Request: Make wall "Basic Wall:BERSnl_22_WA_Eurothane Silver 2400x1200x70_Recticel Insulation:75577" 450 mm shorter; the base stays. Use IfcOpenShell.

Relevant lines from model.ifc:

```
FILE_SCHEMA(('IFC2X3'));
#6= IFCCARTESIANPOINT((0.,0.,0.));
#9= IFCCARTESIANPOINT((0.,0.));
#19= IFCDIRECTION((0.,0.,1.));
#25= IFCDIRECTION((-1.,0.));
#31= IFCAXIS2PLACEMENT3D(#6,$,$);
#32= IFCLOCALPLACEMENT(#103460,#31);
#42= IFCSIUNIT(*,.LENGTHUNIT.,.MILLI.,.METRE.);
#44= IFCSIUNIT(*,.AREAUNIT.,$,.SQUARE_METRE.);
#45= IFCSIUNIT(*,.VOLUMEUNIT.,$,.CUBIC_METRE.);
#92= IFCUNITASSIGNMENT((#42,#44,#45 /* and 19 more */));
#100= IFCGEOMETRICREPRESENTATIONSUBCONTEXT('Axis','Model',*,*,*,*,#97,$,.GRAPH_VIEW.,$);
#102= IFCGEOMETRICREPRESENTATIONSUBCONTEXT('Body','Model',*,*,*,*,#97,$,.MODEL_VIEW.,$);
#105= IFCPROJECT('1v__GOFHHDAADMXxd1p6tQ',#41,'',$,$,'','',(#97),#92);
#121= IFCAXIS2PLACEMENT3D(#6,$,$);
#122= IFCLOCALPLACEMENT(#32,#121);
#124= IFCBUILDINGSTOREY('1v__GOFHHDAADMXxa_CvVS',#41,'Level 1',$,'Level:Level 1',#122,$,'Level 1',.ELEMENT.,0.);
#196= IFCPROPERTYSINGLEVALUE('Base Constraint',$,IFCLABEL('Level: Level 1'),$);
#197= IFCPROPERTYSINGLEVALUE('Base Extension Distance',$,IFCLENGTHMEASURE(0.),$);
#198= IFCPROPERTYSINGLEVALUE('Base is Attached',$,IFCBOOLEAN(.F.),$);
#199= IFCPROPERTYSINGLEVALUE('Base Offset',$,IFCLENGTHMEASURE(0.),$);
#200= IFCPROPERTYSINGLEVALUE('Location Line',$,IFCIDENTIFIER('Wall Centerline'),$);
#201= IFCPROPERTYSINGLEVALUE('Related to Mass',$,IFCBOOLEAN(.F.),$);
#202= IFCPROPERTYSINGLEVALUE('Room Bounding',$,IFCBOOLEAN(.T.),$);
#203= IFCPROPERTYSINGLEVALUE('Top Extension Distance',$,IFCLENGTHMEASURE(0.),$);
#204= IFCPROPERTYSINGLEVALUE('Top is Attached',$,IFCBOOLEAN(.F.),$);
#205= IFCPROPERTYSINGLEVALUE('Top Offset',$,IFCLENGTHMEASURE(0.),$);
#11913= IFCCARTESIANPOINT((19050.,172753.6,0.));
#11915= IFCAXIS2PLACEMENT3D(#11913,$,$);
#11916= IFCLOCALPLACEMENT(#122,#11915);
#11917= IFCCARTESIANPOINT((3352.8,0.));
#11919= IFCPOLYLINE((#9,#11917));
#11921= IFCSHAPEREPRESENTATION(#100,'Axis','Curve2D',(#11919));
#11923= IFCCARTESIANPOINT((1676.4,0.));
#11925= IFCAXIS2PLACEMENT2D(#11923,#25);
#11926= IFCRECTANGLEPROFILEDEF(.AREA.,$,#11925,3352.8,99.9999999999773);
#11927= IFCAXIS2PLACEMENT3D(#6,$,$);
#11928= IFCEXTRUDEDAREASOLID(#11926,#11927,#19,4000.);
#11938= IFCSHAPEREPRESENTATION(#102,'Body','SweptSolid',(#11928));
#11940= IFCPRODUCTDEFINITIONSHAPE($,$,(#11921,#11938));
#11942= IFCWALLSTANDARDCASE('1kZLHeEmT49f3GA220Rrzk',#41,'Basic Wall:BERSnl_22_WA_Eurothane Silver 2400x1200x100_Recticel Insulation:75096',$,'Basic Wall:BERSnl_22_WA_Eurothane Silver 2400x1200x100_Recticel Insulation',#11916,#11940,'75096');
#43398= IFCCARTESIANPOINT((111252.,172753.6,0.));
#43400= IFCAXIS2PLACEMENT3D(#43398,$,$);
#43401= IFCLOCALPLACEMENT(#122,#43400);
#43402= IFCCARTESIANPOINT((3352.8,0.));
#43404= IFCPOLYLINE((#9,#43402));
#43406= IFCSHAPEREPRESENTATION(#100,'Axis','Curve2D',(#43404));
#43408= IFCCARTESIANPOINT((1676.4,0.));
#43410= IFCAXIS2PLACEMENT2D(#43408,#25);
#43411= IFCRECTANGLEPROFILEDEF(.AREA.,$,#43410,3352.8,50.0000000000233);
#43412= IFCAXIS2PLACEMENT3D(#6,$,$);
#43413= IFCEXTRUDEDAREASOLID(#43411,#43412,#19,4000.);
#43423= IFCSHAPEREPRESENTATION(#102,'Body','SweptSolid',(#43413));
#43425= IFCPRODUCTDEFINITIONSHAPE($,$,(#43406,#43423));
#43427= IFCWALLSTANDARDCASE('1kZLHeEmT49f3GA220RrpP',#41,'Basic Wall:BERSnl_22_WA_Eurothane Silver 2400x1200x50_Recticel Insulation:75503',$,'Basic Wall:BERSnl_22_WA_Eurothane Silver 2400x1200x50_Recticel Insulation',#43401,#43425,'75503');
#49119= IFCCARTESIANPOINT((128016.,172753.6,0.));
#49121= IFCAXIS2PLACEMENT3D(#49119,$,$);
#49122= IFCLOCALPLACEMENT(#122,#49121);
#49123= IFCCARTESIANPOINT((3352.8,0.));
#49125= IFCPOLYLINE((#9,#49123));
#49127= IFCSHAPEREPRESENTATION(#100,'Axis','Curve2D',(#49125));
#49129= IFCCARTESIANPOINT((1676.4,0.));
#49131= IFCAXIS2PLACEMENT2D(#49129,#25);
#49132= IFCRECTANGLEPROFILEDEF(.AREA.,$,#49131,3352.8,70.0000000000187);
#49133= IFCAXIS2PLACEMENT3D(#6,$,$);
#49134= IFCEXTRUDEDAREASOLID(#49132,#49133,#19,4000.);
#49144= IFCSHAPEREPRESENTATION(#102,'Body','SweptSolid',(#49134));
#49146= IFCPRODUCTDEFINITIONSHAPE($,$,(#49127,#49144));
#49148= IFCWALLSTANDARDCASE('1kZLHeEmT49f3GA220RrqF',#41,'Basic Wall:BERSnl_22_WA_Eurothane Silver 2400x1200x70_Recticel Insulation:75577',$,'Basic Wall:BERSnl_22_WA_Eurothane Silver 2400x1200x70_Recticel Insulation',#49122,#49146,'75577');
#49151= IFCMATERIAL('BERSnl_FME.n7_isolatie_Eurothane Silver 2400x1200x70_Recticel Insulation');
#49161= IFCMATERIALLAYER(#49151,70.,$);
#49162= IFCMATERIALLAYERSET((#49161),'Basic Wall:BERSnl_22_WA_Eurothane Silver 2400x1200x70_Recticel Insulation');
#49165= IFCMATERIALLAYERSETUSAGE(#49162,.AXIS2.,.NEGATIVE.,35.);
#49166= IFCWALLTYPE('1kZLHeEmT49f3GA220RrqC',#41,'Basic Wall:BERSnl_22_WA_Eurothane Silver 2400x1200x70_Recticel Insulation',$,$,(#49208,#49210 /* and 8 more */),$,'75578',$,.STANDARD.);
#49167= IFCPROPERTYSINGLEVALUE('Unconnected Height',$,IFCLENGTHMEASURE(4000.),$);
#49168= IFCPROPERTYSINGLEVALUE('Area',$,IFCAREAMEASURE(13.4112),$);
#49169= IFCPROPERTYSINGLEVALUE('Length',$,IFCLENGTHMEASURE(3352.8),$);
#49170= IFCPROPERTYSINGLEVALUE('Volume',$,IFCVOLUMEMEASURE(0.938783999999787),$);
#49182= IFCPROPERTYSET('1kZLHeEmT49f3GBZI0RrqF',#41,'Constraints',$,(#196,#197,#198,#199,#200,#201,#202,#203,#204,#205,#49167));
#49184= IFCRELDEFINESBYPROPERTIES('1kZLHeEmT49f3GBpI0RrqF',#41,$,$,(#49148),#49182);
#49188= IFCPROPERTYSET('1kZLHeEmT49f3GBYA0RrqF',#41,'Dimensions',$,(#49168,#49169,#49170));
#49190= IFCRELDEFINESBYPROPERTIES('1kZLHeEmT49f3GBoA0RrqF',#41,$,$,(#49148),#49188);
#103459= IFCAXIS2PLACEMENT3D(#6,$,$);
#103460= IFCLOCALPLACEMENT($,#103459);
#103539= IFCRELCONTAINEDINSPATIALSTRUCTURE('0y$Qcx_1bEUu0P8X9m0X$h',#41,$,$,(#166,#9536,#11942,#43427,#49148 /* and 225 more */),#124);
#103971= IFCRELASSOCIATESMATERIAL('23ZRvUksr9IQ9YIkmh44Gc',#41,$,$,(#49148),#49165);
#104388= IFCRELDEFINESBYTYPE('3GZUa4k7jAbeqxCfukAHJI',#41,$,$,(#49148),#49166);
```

```python
import ifcopenshell
import ifcopenshell.api.pset
import ifcopenshell.geom
import ifcopenshell.util.element
import ifcopenshell.util.representation
import ifcopenshell.util.shape
import ifcopenshell.util.unit

model = ifcopenshell.open("model.ifc")
unit_scale = ifcopenshell.util.unit.calculate_unit_scale(model)
area_scale = ifcopenshell.util.unit.calculate_unit_scale(model, "AREAUNIT")
volume_scale = ifcopenshell.util.unit.calculate_unit_scale(model, "VOLUMEUNIT")
settings = ifcopenshell.geom.settings()


def volume(element):
    """Net volume in cubic metres, openings subtracted."""
    shape = ifcopenshell.geom.create_shape(settings, element)
    return ifcopenshell.util.shape.get_volume(shape.geometry)


wall = model.by_id(49148)
before = volume(wall)

body = ifcopenshell.util.representation.get_representation(wall, "Model", "Body")
solid = body.Items[0]
old_height = solid.Depth
solid.Depth -= 0.45 / unit_scale
after = volume(wall)
thickness = 0.07  # wall thickness in metres

# Update the stored height, areas and volumes.
pset = model.by_id(ifcopenshell.util.element.get_pset(wall, "Constraints", should_inherit=False)["id"])
ifcopenshell.api.pset.edit_pset(model, pset=pset, properties={
    "Unconnected Height": model.create_entity("IfcLengthMeasure", solid.Depth),
})
pset = model.by_id(ifcopenshell.util.element.get_pset(wall, "Dimensions", should_inherit=False)["id"])
ifcopenshell.api.pset.edit_pset(model, pset=pset, properties={
    "Area": model.create_entity("IfcAreaMeasure", after / thickness / area_scale),
    "Volume": model.create_entity("IfcVolumeMeasure", after / volume_scale),
})

print(f"height {old_height:g} -> {solid.Depth:g}, volume {before:.3f} -> {after:.3f} m3")

model.write("model_updated.ifc")
```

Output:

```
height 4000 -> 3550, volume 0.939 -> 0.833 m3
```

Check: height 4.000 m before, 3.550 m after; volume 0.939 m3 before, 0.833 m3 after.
